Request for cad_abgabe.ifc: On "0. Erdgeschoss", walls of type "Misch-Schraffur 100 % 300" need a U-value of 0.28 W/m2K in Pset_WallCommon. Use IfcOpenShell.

First a look at what the model holds.

```python
import ifcopenshell
import ifcopenshell.util.element

model = ifcopenshell.open("cad_abgabe.ifc")
print(model.schema)
storey = next(s for s in model.by_type("IfcBuildingStorey") if s.Name == "0. Erdgeschoss")
walls = [e for e in ifcopenshell.util.element.get_decomposition(storey) if e.is_a("IfcWall")]
seen = {}
for e in walls:
    element_type = ifcopenshell.util.element.get_type(e)
    key = (element_type.Name if element_type != e and element_type else None, ifcopenshell.util.element.get_pset(e, "Pset_WallCommon", "ThermalTransmittance"))
    seen[key] = seen.get(key, 0) + 1
for (name, value), count in sorted(seen.items(), key=str):
    print(count, "x", name, "|", value)
```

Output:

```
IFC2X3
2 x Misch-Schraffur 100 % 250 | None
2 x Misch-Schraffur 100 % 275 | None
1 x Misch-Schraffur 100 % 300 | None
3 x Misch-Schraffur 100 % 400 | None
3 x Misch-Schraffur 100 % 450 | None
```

```python
import ifcopenshell
import ifcopenshell.api.pset
import ifcopenshell.util.element

model = ifcopenshell.open("cad_abgabe.ifc")

storey = next(s for s in model.by_type("IfcBuildingStorey") if s.Name == "0. Erdgeschoss")
walls = [e for e in ifcopenshell.util.element.get_decomposition(storey) if e.is_a("IfcWall")]

count = 0
for e in walls:
    element_type = ifcopenshell.util.element.get_type(e)
    if element_type in (None, e) or element_type.Name != "Misch-Schraffur 100 % 300":
        continue
    # add_pset returns the element's existing set when there is one.
    pset = ifcopenshell.api.pset.add_pset(model, product=e, name="Pset_WallCommon")
    ifcopenshell.api.pset.edit_pset(model, pset=pset, properties={"ThermalTransmittance": 0.28})
    count += 1

print(count, "walls updated")

model.write("cad_abgabe-out.ifc")
```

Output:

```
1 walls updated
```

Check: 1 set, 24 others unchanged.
